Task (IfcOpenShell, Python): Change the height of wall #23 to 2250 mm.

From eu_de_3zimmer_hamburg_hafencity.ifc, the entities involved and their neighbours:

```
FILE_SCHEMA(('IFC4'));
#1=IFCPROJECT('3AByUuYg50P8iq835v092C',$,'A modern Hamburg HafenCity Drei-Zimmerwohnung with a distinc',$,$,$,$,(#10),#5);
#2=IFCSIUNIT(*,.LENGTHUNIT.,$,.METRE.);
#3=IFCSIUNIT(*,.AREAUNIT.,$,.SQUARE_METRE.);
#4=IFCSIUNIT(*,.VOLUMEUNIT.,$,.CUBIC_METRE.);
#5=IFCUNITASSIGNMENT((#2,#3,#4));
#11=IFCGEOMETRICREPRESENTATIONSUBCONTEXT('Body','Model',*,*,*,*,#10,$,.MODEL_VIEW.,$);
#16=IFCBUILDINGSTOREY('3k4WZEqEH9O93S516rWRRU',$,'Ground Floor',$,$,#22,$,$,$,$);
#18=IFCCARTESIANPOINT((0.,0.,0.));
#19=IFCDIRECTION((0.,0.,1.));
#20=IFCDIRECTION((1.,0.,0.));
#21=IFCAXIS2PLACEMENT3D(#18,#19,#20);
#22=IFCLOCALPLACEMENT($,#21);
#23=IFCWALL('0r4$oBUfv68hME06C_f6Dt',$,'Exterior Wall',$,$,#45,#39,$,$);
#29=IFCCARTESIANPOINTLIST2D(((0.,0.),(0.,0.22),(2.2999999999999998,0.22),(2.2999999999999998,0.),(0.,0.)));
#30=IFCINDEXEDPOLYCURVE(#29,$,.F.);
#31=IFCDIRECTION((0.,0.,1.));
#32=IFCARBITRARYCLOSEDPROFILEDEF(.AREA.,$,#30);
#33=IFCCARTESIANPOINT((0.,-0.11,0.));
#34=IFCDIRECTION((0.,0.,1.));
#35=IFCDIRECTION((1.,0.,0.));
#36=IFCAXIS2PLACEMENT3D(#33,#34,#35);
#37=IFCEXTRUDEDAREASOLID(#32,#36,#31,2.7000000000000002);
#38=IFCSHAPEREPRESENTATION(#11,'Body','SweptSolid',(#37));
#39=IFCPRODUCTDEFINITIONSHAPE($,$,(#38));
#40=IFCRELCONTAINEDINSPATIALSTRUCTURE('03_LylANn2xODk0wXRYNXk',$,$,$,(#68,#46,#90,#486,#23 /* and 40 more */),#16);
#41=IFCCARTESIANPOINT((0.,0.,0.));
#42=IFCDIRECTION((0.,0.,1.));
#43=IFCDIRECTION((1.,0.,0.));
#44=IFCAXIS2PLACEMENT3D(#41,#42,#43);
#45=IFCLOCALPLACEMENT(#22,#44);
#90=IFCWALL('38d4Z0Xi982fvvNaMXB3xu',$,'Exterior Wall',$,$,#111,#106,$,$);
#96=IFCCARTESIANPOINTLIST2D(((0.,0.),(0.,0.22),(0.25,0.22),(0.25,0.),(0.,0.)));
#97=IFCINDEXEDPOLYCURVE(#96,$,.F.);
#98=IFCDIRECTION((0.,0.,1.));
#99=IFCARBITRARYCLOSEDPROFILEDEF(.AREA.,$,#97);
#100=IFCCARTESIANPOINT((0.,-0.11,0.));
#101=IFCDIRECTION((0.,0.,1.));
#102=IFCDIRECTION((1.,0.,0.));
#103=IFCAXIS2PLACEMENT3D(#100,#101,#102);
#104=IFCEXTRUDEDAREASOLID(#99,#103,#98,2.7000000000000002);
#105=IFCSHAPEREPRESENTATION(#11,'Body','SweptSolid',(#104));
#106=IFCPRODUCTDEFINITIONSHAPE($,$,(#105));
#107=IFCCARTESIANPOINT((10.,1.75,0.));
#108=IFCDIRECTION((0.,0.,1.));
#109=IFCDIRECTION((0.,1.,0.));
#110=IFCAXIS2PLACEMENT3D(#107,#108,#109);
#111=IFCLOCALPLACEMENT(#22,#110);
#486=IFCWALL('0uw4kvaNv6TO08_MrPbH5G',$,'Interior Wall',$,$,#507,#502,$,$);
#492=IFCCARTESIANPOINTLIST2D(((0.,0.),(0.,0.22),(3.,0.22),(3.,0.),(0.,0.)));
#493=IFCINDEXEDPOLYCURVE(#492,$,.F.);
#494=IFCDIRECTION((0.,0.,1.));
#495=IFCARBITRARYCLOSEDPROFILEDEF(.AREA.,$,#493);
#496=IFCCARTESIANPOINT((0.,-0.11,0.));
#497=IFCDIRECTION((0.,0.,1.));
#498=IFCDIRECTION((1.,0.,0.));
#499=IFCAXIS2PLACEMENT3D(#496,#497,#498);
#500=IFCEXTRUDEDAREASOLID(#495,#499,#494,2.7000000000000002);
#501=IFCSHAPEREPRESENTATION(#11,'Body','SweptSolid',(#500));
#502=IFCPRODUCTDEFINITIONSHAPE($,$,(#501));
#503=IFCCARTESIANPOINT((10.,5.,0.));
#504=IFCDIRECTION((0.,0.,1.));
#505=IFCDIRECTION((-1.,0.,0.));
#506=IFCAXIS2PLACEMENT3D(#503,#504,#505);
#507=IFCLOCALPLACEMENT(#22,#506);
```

```python
import ifcopenshell
import ifcopenshell.geom
import ifcopenshell.util.representation
import ifcopenshell.util.shape
import ifcopenshell.util.unit

model = ifcopenshell.open("eu_de_3zimmer_hamburg_hafencity.ifc")
unit_scale = ifcopenshell.util.unit.calculate_unit_scale(model)
settings = ifcopenshell.geom.settings()


def volume(element):
    """Net volume in cubic metres, openings subtracted."""
    shape = ifcopenshell.geom.create_shape(settings, element)
    return ifcopenshell.util.shape.get_volume(shape.geometry)


wall = model.by_guid("0r4$oBUfv68hME06C_f6Dt")
before = volume(wall)

body = ifcopenshell.util.representation.get_representation(wall, "Model", "Body")
solid = body.Items[0]
old_height = solid.Depth
solid.Depth = 2.25 / unit_scale
after = volume(wall)

print(f"height {old_height:g} -> {solid.Depth:g}, volume {before:.3f} -> {after:.3f} m3")

model.write("eu_de_3zimmer_hamburg_hafencity_edited.ifc")
```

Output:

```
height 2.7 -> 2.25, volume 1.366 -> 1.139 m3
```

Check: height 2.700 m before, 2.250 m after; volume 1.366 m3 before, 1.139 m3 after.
